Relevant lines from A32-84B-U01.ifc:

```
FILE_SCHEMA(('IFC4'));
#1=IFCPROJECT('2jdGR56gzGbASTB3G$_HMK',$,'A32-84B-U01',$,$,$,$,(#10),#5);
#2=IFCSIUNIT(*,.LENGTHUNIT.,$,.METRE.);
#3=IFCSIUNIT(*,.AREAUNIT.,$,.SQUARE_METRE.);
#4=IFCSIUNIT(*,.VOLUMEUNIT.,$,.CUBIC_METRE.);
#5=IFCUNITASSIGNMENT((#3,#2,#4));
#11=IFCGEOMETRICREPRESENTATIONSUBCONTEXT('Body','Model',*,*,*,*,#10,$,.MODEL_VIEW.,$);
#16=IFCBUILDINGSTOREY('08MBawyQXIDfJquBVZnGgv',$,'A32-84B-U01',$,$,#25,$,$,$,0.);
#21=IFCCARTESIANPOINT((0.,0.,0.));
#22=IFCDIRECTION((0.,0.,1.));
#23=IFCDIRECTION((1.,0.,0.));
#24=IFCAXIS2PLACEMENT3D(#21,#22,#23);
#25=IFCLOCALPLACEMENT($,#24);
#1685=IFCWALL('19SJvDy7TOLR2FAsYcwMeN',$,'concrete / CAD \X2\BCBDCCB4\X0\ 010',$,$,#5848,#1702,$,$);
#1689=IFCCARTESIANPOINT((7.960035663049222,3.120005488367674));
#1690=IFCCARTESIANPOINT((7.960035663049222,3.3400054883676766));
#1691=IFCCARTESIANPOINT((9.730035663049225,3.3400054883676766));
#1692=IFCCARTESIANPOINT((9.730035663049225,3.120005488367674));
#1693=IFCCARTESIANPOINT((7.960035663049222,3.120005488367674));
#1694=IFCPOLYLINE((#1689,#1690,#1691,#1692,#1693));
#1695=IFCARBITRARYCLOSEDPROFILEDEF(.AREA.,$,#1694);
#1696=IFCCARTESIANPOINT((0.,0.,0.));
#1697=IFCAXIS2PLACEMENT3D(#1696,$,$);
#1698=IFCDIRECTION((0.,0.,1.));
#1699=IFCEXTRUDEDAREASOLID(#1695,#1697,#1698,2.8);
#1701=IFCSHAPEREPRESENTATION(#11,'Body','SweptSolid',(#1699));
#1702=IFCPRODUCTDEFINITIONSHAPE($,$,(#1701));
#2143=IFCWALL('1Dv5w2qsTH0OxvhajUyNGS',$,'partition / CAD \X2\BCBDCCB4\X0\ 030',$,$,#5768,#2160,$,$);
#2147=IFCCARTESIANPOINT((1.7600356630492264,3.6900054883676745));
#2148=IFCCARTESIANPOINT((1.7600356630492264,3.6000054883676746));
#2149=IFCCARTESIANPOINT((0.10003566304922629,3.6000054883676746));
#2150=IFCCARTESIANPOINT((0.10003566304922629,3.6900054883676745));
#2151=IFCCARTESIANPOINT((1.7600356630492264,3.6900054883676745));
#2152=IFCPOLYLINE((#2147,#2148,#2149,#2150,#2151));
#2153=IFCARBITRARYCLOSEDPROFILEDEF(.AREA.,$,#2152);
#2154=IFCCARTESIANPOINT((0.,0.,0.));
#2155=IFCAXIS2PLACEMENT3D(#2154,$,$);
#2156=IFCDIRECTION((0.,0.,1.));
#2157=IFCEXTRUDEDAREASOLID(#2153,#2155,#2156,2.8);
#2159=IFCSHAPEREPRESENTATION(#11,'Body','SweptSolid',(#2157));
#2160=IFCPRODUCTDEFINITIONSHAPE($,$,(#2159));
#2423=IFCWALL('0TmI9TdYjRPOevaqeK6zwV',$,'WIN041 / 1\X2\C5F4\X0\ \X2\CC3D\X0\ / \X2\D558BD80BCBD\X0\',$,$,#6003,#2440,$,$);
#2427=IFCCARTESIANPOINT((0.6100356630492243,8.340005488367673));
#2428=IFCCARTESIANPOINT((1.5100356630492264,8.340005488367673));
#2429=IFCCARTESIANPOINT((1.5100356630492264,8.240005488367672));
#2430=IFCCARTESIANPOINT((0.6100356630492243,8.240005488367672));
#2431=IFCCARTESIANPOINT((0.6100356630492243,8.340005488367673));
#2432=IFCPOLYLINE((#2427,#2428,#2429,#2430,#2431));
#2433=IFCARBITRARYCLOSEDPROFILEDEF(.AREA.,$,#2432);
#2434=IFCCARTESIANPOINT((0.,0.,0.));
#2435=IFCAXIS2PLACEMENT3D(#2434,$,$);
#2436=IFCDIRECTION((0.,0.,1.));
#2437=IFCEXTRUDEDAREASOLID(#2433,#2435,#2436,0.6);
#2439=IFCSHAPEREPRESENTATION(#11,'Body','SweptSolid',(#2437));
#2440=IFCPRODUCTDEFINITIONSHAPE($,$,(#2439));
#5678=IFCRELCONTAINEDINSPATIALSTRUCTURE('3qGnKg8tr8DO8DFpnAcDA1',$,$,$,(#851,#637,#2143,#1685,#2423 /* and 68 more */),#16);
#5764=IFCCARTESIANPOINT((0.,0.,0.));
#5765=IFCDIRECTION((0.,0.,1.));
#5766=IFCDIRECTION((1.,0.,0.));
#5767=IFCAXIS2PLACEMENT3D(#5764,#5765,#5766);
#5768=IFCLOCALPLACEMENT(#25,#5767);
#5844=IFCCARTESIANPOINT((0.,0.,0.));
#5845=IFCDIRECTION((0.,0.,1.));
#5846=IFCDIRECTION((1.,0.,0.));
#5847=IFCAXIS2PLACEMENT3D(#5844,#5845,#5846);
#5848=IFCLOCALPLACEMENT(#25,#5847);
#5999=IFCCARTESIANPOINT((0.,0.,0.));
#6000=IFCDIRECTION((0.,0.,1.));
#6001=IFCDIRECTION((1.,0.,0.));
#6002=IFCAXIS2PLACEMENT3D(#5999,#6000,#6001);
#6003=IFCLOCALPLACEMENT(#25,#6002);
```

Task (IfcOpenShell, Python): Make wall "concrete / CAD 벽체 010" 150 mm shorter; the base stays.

```python
import ifcopenshell
import ifcopenshell.geom
import ifcopenshell.util.representation
import ifcopenshell.util.shape
import ifcopenshell.util.unit

model = ifcopenshell.open("A32-84B-U01.ifc")
unit_scale = ifcopenshell.util.unit.calculate_unit_scale(model)
settings = ifcopenshell.geom.settings()


def volume(element):
    """Net volume in cubic metres, openings subtracted."""
    shape = ifcopenshell.geom.create_shape(settings, element)
    return ifcopenshell.util.shape.get_volume(shape.geometry)


wall = model.by_guid("19SJvDy7TOLR2FAsYcwMeN")
before = volume(wall)

body = ifcopenshell.util.representation.get_representation(wall, "Model", "Body")
solid = body.Items[0]
old_height = solid.Depth
solid.Depth -= 0.15 / unit_scale
after = volume(wall)

print(f"height {old_height:g} -> {solid.Depth:g}, volume {before:.3f} -> {after:.3f} m3")

model.write("A32-84B-U01_updated.ifc")
```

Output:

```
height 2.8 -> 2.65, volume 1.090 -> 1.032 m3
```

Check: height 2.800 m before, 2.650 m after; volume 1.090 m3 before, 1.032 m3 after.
